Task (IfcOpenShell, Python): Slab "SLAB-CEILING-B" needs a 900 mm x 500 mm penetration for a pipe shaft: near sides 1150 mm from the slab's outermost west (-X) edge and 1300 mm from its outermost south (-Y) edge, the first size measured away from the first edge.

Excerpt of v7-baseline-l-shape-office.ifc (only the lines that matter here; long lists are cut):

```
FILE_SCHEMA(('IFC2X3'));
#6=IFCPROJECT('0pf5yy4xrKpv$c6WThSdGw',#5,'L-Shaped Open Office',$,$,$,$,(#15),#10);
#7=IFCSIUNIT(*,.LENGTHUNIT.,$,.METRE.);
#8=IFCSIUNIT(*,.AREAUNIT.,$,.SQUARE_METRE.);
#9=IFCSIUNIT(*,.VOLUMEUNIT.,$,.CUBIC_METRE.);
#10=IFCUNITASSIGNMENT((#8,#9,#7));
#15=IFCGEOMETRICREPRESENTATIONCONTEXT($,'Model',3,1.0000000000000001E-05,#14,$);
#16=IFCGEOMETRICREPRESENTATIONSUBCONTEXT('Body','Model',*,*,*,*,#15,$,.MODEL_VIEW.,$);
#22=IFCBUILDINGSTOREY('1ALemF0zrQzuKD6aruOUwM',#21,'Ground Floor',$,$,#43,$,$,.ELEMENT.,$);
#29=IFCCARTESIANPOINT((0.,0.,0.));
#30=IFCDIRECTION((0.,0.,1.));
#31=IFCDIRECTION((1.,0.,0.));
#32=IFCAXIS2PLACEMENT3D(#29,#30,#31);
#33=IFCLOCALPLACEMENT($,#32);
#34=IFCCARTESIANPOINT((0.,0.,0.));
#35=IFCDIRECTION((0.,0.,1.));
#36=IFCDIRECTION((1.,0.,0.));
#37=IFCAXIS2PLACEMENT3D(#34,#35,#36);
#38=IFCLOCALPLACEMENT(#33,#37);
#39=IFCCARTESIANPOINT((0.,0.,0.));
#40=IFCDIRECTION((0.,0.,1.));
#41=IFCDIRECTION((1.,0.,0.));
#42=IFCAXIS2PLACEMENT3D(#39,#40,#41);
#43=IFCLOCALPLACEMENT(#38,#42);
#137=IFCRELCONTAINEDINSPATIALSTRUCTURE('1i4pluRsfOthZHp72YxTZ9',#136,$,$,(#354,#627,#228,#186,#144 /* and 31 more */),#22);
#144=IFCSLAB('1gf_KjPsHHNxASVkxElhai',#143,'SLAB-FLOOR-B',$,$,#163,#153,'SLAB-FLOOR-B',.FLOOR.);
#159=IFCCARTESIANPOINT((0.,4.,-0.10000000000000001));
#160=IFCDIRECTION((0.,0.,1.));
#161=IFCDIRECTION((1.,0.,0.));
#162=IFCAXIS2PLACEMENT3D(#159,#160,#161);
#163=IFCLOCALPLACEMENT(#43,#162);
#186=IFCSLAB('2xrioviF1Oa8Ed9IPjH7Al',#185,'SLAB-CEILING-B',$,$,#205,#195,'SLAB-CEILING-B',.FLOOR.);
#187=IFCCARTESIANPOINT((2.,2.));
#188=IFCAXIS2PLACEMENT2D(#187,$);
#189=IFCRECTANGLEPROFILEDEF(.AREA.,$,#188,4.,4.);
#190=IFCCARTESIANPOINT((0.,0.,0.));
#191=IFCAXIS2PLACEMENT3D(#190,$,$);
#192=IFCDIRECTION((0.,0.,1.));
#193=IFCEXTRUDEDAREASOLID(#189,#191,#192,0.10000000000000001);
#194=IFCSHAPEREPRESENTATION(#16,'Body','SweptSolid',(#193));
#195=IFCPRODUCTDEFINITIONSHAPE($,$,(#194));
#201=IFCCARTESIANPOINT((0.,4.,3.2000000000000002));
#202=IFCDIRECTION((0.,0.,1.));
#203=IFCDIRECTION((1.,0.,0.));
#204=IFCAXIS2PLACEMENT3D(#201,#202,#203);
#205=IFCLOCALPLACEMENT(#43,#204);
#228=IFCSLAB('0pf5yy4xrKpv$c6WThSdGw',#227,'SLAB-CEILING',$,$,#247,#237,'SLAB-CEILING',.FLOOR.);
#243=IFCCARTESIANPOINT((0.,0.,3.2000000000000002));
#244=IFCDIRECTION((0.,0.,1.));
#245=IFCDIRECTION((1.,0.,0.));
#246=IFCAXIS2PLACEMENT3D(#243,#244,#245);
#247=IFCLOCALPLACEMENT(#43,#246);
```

```python
import numpy as np
import ifcopenshell
import ifcopenshell.api.feature
import ifcopenshell.api.geometry
import ifcopenshell.api.root
import ifcopenshell.geom
import ifcopenshell.util.placement
import ifcopenshell.util.representation
import ifcopenshell.util.shape
import ifcopenshell.util.unit

model = ifcopenshell.open("v7-baseline-l-shape-office.ifc")
unit_scale = ifcopenshell.util.unit.calculate_unit_scale(model)
settings = ifcopenshell.geom.settings()


def volume(element):
    """Net volume in cubic metres, openings subtracted."""
    shape = ifcopenshell.geom.create_shape(settings, element)
    return ifcopenshell.util.shape.get_volume(shape.geometry)


slab = model.by_id(186)
before = volume(slab)

# Extent in the slab's own axes, in metres. The edges named are its -X and -Y sides.
slab_shape = ifcopenshell.geom.create_shape(settings, slab)
vertices = ifcopenshell.util.shape.get_vertices(slab_shape.geometry)
x_min, y_min, bottom = vertices.min(axis=0)
top = vertices[:, 2].max()

opening = ifcopenshell.api.root.create_entity(model, ifc_class="IfcOpeningElement", name="Pipe shaft opening")
context = ifcopenshell.util.representation.get_context(model, "Model", "Body", "MODEL_VIEW")
width, depth = 0.9, 0.5
outline = [(0.0, 0.0), (width, 0.0), (width, depth), (0.0, depth), (0.0, 0.0)]
# Overshoot both faces by 50 mm so the cut is clean.
shape = ifcopenshell.api.geometry.add_slab_representation(
    model, context=context, depth=top - bottom + 0.1, polyline=outline
)
ifcopenshell.api.geometry.assign_representation(model, product=opening, representation=shape)

matrix = ifcopenshell.util.placement.get_local_placement(slab.ObjectPlacement)
matrix[:, 3] = matrix @ np.append(np.array([x_min + 1.15, y_min + 1.3, bottom - 0.05]) / unit_scale, 1.0)
ifcopenshell.api.geometry.edit_object_placement(model, product=opening, matrix=matrix, is_si=False)
ifcopenshell.api.feature.add_feature(model, feature=opening, element=slab)

after = volume(slab)

print(f"slab volume {before:.3f} -> {after:.3f} m3")

model.write("v7-baseline-l-shape-office_rev.ifc")
```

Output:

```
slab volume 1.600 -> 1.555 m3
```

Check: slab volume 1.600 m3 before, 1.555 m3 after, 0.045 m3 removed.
